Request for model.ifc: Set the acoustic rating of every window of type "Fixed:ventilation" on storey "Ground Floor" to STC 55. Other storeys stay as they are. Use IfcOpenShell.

First a look at what the model holds.

```python
import ifcopenshell
import ifcopenshell.util.element

model = ifcopenshell.open("model.ifc")
print(model.schema)
storey = next(s for s in model.by_type("IfcBuildingStorey") if s.Name == "Ground Floor")
windows = [e for e in ifcopenshell.util.element.get_decomposition(storey) if e.is_a("IfcWindow")]
seen = {}
for e in windows:
    element_type = ifcopenshell.util.element.get_type(e)
    key = (element_type.Name if element_type != e and element_type else None, ifcopenshell.util.element.get_pset(e, "Pset_WindowCommon", "AcousticRating"))
    seen[key] = seen.get(key, 0) + 1
for (name, value), count in sorted(seen.items(), key=str):
    print(count, "x", name, "|", value)
```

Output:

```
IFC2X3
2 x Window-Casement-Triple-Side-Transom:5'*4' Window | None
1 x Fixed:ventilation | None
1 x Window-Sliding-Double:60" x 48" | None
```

```python
import ifcopenshell
import ifcopenshell.api.pset
import ifcopenshell.util.element

model = ifcopenshell.open("model.ifc")

storey = next(s for s in model.by_type("IfcBuildingStorey") if s.Name == "Ground Floor")
windows = [e for e in ifcopenshell.util.element.get_decomposition(storey) if e.is_a("IfcWindow")]

count = 0
for e in windows:
    element_type = ifcopenshell.util.element.get_type(e)
    if element_type in (None, e) or element_type.Name != "Fixed:ventilation":
        continue
    # add_pset returns the element's existing set when there is one.
    pset = ifcopenshell.api.pset.add_pset(model, product=e, name="Pset_WindowCommon")
    ifcopenshell.api.pset.edit_pset(model, pset=pset, properties={"AcousticRating": "STC 55"})
    count += 1

print(count, "windows updated")

model.write("model_rev.ifc")
```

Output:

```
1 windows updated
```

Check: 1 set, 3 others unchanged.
